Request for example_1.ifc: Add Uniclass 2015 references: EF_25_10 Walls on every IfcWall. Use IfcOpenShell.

First a look at what the model holds.

```python
import ifcopenshell

model = ifcopenshell.open("example_1.ifc")
print(model.schema)
print("classifications:", [c.Name for c in model.by_type("IfcClassification")])
for ifc_class in ("IfcDoor", "IfcRoof", "IfcStair", "IfcWall", "IfcWindow"):
    print(ifc_class, len(model.by_type(ifc_class)))
```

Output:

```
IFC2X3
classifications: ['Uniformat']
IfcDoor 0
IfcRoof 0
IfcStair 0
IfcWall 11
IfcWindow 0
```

```python
import ifcopenshell
import ifcopenshell.api.classification

model = ifcopenshell.open("example_1.ifc")

# IFC2X3 requires Source and Edition and has no link from the project to the system.
system = model.create_entity("IfcClassification", Source="NBS", Edition="2015", Name="Uniclass 2015")

codes = {
    "IfcWall": ("EF_25_10", "Walls"),
}
for ifc_class, (code, name) in codes.items():
    products = model.by_type(ifc_class)
    ifcopenshell.api.classification.add_reference(
        model, products=products, classification=system, identification=code, name=name
    )
    print(code, len(products))

model.write("example_1_edited.ifc")
```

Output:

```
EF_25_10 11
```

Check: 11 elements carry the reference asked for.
